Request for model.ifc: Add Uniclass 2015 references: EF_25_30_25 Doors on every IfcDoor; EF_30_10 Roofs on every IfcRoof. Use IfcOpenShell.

First a look at what the model holds.

```python
import ifcopenshell

model = ifcopenshell.open("model.ifc")
print(model.schema)
print("classifications:", [c.Name for c in model.by_type("IfcClassification")])
for ifc_class in ("IfcDoor", "IfcRoof", "IfcStair", "IfcWall", "IfcWindow"):
    print(ifc_class, len(model.by_type(ifc_class)))
```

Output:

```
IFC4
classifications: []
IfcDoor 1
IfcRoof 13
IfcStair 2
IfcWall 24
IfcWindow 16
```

```python
import ifcopenshell
import ifcopenshell.api.classification

model = ifcopenshell.open("model.ifc")

system = ifcopenshell.api.classification.add_classification(model, classification="Uniclass 2015")

codes = {
    "IfcDoor": ("EF_25_30_25", "Doors"),
    "IfcRoof": ("EF_30_10", "Roofs"),
}
for ifc_class, (code, name) in codes.items():
    products = model.by_type(ifc_class)
    ifcopenshell.api.classification.add_reference(
        model, products=products, classification=system, identification=code, name=name
    )
    print(code, len(products))

model.write("model_edited.ifc")
```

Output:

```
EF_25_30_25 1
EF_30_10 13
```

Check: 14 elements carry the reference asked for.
